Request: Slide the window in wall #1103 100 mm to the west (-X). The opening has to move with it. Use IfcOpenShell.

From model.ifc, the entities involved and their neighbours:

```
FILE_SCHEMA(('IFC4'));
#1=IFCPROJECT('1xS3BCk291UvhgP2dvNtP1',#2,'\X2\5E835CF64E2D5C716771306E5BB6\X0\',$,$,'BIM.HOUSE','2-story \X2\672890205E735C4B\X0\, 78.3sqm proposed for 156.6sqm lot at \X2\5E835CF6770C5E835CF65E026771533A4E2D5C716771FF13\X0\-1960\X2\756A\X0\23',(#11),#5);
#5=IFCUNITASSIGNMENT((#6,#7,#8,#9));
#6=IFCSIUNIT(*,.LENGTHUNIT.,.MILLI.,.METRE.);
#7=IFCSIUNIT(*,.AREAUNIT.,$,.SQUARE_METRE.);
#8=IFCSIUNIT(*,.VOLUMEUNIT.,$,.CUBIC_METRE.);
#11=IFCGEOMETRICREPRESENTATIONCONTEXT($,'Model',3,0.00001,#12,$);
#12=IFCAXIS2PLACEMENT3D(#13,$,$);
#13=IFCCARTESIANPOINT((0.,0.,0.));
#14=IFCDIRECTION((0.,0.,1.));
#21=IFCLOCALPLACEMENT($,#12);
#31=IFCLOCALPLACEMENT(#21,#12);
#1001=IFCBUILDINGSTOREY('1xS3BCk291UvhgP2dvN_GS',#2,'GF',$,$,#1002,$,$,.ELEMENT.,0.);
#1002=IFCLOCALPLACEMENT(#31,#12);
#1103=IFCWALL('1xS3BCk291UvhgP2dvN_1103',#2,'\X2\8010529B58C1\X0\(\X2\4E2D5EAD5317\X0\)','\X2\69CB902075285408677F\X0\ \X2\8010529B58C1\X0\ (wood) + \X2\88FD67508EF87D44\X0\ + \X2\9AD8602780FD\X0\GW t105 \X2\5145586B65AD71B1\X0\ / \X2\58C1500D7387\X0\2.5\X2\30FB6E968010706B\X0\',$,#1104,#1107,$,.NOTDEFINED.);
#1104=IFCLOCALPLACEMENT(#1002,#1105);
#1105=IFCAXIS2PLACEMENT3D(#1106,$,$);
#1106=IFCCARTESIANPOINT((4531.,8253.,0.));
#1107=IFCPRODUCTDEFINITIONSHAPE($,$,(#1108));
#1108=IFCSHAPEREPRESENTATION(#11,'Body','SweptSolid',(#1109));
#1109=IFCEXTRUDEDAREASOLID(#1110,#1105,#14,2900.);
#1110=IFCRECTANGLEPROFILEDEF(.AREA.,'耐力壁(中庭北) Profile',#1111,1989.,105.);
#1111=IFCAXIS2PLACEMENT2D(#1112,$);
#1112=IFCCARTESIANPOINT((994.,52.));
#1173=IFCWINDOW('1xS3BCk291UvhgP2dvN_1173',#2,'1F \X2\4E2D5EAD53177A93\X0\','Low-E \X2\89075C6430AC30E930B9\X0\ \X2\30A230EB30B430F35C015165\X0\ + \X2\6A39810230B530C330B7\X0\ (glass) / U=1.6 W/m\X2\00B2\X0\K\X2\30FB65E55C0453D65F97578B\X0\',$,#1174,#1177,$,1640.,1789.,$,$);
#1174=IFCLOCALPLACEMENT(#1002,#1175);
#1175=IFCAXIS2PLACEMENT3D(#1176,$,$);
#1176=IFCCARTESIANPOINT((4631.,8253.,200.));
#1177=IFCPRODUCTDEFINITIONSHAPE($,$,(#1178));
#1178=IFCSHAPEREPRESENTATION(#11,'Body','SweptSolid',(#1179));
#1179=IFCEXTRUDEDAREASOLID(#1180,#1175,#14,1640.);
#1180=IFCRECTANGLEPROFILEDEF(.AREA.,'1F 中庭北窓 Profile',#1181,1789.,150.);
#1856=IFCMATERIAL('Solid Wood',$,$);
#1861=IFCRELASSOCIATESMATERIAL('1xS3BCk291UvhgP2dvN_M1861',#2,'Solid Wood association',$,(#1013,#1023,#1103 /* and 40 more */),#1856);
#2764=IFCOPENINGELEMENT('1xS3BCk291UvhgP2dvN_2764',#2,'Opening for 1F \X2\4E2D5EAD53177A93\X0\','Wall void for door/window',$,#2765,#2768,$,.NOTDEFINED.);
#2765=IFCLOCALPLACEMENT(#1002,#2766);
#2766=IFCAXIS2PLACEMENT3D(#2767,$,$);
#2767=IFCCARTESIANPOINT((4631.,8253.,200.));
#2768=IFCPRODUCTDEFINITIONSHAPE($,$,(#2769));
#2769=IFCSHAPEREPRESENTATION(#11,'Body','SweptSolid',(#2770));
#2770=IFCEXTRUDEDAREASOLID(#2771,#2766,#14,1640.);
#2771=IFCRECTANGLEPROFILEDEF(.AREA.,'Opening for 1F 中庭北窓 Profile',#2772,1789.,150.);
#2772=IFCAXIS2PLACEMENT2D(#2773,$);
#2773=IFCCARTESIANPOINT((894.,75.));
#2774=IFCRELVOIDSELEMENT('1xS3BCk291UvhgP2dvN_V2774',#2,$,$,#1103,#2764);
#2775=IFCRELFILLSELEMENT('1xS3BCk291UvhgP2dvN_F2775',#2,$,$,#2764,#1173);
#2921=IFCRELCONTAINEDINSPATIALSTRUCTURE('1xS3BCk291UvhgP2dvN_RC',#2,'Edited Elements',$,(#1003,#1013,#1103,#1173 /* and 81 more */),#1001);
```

```python
import ifcopenshell
import ifcopenshell.api.geometry
import ifcopenshell.util.placement
import ifcopenshell.util.unit

model = ifcopenshell.open("model.ifc")
unit_scale = ifcopenshell.util.unit.calculate_unit_scale(model)

window = model.by_id(1173)
opening = window.FillsVoids[0].RelatingOpeningElement
wall = opening.VoidsElements[0].RelatingBuildingElement

wall_matrix = ifcopenshell.util.placement.get_local_placement(wall.ObjectPlacement)
shift = wall_matrix[:3, 0] * -0.1 / unit_scale
before = ifcopenshell.util.placement.get_local_placement(window.ObjectPlacement)[:3, 3].copy()

# The window is not placed relative to its opening, so move both.
for product in (opening, window):
    matrix = ifcopenshell.util.placement.get_local_placement(product.ObjectPlacement)
    matrix[:3, 3] += shift
    ifcopenshell.api.geometry.edit_object_placement(model, product=product, matrix=matrix, is_si=False)

after = ifcopenshell.util.placement.get_local_placement(window.ObjectPlacement)[:3, 3]
print("window moved by", (after - before).round(3) + 0.0)

model.write("model_edited.ifc")
```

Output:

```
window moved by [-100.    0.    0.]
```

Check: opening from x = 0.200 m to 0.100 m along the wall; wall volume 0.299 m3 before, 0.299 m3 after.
